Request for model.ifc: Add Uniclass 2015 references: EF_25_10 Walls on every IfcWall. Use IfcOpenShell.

First a look at what the model holds.

```python
import ifcopenshell

model = ifcopenshell.open("model.ifc")
print(model.schema)
print("classifications:", [c.Name for c in model.by_type("IfcClassification")])
for ifc_class in ("IfcDoor", "IfcRoof", "IfcStair", "IfcWall", "IfcWindow"):
    print(ifc_class, len(model.by_type(ifc_class)))
```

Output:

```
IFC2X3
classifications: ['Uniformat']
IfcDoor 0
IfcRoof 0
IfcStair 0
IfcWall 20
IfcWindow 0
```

```python
import ifcopenshell
import ifcopenshell.api.classification

model = ifcopenshell.open("model.ifc")

# IFC2X3 requires Source and Edition and has no link from the project to the system.
system = model.create_entity("IfcClassification", Source="NBS", Edition="2015", Name="Uniclass 2015")

codes = {
    "IfcWall": ("EF_25_10", "Walls"),
}
for ifc_class, (code, name) in codes.items():
    products = model.by_type(ifc_class)
    ifcopenshell.api.classification.add_reference(
        model, products=products, classification=system, identification=code, name=name
    )
    print(code, len(products))

model.write("model_updated.ifc")
```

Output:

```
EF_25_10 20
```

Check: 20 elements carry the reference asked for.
